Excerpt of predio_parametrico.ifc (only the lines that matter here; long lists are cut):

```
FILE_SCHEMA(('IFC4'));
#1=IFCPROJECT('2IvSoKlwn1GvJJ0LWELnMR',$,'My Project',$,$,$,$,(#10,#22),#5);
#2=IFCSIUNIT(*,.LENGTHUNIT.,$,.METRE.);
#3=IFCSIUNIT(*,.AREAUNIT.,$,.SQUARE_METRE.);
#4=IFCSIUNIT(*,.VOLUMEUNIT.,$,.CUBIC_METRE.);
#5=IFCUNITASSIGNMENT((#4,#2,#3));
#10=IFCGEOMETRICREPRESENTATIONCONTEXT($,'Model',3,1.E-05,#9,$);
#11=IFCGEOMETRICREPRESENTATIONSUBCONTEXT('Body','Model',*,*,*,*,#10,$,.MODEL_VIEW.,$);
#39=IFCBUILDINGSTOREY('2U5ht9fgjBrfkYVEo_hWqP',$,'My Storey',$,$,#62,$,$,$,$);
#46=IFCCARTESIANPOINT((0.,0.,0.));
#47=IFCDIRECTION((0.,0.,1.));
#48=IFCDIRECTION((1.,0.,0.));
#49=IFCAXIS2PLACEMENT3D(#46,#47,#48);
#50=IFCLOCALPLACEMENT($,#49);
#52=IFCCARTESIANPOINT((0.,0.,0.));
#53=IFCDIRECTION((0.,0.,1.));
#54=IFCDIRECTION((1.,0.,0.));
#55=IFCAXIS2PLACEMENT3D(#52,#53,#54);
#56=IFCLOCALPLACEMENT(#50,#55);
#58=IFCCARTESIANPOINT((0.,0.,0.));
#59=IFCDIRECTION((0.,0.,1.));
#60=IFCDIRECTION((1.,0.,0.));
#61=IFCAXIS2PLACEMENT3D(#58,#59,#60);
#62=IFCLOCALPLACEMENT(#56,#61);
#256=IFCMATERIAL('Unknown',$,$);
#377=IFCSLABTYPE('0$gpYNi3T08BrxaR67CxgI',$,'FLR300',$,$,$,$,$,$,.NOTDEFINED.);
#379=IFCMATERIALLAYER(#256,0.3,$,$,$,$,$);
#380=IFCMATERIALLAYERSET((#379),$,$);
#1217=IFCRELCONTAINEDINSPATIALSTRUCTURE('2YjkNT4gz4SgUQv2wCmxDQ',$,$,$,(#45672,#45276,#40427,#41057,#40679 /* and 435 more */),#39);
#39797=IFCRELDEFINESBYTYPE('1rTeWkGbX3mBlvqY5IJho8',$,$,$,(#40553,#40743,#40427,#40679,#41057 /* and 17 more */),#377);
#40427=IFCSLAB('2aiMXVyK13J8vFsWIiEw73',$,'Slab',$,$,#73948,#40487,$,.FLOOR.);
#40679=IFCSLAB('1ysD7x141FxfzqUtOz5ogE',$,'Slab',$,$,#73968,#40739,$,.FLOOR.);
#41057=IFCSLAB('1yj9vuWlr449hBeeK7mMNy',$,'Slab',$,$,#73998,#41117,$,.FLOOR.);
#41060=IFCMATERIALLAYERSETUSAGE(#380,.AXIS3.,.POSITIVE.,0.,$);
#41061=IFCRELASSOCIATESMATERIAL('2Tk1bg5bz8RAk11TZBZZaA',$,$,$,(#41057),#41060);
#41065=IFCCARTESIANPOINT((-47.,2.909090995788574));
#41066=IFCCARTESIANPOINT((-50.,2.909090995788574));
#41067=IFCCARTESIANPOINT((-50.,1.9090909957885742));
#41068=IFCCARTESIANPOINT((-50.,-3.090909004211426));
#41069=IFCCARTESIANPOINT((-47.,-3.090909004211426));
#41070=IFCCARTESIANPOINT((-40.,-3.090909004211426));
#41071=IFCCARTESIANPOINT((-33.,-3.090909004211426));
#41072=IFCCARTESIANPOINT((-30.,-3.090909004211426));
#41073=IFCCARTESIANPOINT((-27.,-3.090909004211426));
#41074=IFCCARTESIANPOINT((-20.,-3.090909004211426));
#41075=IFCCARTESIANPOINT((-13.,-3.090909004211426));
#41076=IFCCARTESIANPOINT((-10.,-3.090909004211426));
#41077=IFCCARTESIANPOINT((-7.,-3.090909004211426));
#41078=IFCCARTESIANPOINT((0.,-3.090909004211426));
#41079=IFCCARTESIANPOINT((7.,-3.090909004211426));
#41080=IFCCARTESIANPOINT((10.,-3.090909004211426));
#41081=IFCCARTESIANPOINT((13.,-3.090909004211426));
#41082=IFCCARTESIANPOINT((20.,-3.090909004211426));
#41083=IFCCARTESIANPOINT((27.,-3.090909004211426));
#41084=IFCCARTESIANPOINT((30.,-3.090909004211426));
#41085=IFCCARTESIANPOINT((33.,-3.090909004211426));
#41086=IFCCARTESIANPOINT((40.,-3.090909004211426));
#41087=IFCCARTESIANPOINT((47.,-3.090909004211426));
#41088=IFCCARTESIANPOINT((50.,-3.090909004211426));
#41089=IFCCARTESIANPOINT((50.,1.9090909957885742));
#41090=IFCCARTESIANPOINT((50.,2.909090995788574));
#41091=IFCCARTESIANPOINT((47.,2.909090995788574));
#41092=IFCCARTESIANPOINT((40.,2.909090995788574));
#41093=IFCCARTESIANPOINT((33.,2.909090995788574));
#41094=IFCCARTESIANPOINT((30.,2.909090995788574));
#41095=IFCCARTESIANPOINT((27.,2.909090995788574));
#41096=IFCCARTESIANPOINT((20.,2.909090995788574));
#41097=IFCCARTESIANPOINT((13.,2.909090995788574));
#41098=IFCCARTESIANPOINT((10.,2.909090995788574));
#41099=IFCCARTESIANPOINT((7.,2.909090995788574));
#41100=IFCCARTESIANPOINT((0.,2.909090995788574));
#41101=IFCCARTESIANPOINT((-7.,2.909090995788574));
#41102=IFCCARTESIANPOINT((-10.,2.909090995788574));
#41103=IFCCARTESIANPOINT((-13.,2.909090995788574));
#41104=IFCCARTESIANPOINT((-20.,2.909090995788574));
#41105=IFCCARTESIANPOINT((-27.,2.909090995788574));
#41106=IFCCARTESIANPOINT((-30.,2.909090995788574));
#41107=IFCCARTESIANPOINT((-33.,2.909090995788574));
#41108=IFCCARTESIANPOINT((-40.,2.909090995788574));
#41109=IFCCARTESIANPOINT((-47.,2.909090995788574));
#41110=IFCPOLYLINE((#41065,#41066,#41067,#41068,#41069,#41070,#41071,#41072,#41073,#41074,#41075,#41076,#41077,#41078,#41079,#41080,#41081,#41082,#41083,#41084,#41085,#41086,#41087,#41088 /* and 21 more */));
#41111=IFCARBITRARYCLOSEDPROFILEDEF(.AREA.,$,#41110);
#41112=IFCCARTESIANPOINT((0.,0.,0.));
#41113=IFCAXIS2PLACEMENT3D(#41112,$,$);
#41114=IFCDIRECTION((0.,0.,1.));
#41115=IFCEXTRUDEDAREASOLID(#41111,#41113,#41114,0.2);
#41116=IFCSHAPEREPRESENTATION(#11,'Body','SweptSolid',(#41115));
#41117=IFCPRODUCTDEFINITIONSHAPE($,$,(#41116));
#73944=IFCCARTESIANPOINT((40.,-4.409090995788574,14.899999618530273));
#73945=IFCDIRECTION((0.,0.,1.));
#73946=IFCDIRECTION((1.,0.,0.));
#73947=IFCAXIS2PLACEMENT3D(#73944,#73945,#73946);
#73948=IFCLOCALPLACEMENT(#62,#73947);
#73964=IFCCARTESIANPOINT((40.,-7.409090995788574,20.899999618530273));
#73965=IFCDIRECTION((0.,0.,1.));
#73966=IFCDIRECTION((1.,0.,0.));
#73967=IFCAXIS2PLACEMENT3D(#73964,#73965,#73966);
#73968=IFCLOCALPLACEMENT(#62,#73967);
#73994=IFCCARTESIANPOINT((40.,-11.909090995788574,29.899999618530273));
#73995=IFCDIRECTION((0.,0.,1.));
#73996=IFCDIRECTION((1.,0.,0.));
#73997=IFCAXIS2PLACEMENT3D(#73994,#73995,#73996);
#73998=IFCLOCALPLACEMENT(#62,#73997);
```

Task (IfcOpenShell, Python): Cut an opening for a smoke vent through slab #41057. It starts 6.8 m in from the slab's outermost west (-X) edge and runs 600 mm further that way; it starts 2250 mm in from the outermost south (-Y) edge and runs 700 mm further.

```python
import numpy as np
import ifcopenshell
import ifcopenshell.api.feature
import ifcopenshell.api.geometry
import ifcopenshell.api.root
import ifcopenshell.geom
import ifcopenshell.util.placement
import ifcopenshell.util.representation
import ifcopenshell.util.shape
import ifcopenshell.util.unit

model = ifcopenshell.open("predio_parametrico.ifc")
unit_scale = ifcopenshell.util.unit.calculate_unit_scale(model)
settings = ifcopenshell.geom.settings()


def volume(element):
    """Net volume in cubic metres, openings subtracted."""
    shape = ifcopenshell.geom.create_shape(settings, element)
    return ifcopenshell.util.shape.get_volume(shape.geometry)


slab = model.by_guid("1yj9vuWlr449hBeeK7mMNy")
before = volume(slab)

# Extent in the slab's own axes, in metres. The edges named are its -X and -Y sides.
slab_shape = ifcopenshell.geom.create_shape(settings, slab)
vertices = ifcopenshell.util.shape.get_vertices(slab_shape.geometry)
x_min, y_min, bottom = vertices.min(axis=0)
top = vertices[:, 2].max()

opening = ifcopenshell.api.root.create_entity(model, ifc_class="IfcOpeningElement", name="Smoke vent opening", predefined_type="OPENING")
context = ifcopenshell.util.representation.get_context(model, "Model", "Body", "MODEL_VIEW")
width, depth = 0.6, 0.7
outline = [(0.0, 0.0), (width, 0.0), (width, depth), (0.0, depth), (0.0, 0.0)]
# Overshoot both faces by 50 mm so the cut is clean.
shape = ifcopenshell.api.geometry.add_slab_representation(
    model, context=context, depth=top - bottom + 0.1, polyline=outline
)
ifcopenshell.api.geometry.assign_representation(model, product=opening, representation=shape)

matrix = ifcopenshell.util.placement.get_local_placement(slab.ObjectPlacement)
matrix[:, 3] = matrix @ np.append(np.array([x_min + 6.8, y_min + 2.25, bottom - 0.05]) / unit_scale, 1.0)
ifcopenshell.api.geometry.edit_object_placement(model, product=opening, matrix=matrix, is_si=False)
ifcopenshell.api.feature.add_feature(model, feature=opening, element=slab)

after = volume(slab)

print(f"slab volume {before:.3f} -> {after:.3f} m3")

model.write("predio_parametrico_v2.ifc")
```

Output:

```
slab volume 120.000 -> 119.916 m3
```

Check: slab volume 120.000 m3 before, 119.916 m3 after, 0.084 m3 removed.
